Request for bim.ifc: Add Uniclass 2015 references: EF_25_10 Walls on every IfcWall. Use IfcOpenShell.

First a look at what the model holds.

```python
import ifcopenshell

model = ifcopenshell.open("bim.ifc")
print(model.schema)
print("classifications:", [c.Name for c in model.by_type("IfcClassification")])
for ifc_class in ("IfcDoor", "IfcRoof", "IfcStair", "IfcWall", "IfcWindow"):
    print(ifc_class, len(model.by_type(ifc_class)))
```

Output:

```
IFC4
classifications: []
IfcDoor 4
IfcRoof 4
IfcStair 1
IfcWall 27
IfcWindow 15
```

```python
import ifcopenshell
import ifcopenshell.api.classification

model = ifcopenshell.open("bim.ifc")

system = ifcopenshell.api.classification.add_classification(model, classification="Uniclass 2015")

codes = {
    "IfcWall": ("EF_25_10", "Walls"),
}
for ifc_class, (code, name) in codes.items():
    products = model.by_type(ifc_class)
    ifcopenshell.api.classification.add_reference(
        model, products=products, classification=system, identification=code, name=name
    )
    print(code, len(products))

model.write("bim-out.ifc")
```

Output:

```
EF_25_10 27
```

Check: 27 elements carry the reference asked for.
